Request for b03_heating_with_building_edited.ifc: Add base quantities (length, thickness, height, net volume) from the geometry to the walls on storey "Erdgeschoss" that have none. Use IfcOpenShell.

First a look at what the model holds.

```python
import ifcopenshell
import ifcopenshell.util.element
import ifcopenshell.util.unit

model = ifcopenshell.open("b03_heating_with_building_edited.ifc")
print(model.schema)
for unit_type in ("LENGTHUNIT", "AREAUNIT", "VOLUMEUNIT"):
    print(unit_type, ifcopenshell.util.unit.calculate_unit_scale(model, unit_type))
storey = next(s for s in model.by_type("IfcBuildingStorey") if s.Name == "Erdgeschoss")
walls = [e for e in ifcopenshell.util.element.get_decomposition(storey) if e.is_a("IfcWall")]
for e in sorted(walls, key=lambda e: e.id()):
    print(e.id(), e.is_a(), e.Name, list(ifcopenshell.util.element.get_psets(e, qtos_only=True)), sep=" | ")
```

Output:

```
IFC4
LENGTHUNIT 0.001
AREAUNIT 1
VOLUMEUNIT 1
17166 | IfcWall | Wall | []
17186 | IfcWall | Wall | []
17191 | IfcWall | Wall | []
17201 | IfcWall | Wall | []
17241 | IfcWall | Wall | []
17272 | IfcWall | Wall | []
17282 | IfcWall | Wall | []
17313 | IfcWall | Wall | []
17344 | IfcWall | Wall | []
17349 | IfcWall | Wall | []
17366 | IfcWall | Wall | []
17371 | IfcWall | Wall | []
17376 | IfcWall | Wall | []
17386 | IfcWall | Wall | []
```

```python
import ifcopenshell
import ifcopenshell.api.pset
import ifcopenshell.geom
import ifcopenshell.util.element
import ifcopenshell.util.shape
import ifcopenshell.util.unit

model = ifcopenshell.open("b03_heating_with_building_edited.ifc")
unit_scale = ifcopenshell.util.unit.calculate_unit_scale(model)
volume_scale = ifcopenshell.util.unit.calculate_unit_scale(model, "VOLUMEUNIT")
settings = ifcopenshell.geom.settings()

storey = next(s for s in model.by_type("IfcBuildingStorey") if s.Name == "Erdgeschoss")
walls = [e for e in ifcopenshell.util.element.get_decomposition(storey) if e.is_a("IfcWall")]

for e in sorted(walls, key=lambda e: e.id()):
    if ifcopenshell.util.element.get_psets(e, qtos_only=True, should_inherit=False):
        continue
    # Geometry comes back in metres, in the element's own axes.
    shape = ifcopenshell.geom.create_shape(settings, e)
    values = {
        "Length": ifcopenshell.util.shape.get_x(shape.geometry) / unit_scale,
        "Width": ifcopenshell.util.shape.get_y(shape.geometry) / unit_scale,
        "Height": ifcopenshell.util.shape.get_z(shape.geometry) / unit_scale,
        "NetVolume": ifcopenshell.util.shape.get_volume(shape.geometry) / volume_scale,
    }
    qto = ifcopenshell.api.pset.add_qto(model, product=e, name="Qto_WallBaseQuantities")
    ifcopenshell.api.pset.edit_qto(model, qto=qto, properties=values)
    print(e.id(), {k: round(v, 3) for k, v in values.items()})

model.write("b03_heating_with_building_edited_updated.ifc")
```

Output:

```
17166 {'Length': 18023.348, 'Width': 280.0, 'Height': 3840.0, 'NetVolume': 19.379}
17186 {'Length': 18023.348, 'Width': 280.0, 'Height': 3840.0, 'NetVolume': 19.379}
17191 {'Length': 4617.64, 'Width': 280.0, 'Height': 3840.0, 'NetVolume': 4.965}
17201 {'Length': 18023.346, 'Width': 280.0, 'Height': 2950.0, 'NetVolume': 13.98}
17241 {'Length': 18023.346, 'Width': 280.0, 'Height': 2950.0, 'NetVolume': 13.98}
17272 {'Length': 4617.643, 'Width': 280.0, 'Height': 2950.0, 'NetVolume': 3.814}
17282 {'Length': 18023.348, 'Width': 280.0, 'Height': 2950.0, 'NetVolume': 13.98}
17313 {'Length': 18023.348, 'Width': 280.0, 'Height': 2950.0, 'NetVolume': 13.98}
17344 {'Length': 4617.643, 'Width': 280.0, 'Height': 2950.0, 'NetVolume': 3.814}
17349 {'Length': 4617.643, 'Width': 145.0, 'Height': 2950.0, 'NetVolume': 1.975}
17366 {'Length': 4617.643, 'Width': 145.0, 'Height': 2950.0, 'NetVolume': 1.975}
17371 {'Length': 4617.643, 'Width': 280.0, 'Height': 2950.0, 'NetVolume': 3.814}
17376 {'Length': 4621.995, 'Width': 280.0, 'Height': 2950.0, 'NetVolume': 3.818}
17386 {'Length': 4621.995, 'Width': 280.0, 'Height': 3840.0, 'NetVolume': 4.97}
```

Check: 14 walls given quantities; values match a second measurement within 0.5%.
